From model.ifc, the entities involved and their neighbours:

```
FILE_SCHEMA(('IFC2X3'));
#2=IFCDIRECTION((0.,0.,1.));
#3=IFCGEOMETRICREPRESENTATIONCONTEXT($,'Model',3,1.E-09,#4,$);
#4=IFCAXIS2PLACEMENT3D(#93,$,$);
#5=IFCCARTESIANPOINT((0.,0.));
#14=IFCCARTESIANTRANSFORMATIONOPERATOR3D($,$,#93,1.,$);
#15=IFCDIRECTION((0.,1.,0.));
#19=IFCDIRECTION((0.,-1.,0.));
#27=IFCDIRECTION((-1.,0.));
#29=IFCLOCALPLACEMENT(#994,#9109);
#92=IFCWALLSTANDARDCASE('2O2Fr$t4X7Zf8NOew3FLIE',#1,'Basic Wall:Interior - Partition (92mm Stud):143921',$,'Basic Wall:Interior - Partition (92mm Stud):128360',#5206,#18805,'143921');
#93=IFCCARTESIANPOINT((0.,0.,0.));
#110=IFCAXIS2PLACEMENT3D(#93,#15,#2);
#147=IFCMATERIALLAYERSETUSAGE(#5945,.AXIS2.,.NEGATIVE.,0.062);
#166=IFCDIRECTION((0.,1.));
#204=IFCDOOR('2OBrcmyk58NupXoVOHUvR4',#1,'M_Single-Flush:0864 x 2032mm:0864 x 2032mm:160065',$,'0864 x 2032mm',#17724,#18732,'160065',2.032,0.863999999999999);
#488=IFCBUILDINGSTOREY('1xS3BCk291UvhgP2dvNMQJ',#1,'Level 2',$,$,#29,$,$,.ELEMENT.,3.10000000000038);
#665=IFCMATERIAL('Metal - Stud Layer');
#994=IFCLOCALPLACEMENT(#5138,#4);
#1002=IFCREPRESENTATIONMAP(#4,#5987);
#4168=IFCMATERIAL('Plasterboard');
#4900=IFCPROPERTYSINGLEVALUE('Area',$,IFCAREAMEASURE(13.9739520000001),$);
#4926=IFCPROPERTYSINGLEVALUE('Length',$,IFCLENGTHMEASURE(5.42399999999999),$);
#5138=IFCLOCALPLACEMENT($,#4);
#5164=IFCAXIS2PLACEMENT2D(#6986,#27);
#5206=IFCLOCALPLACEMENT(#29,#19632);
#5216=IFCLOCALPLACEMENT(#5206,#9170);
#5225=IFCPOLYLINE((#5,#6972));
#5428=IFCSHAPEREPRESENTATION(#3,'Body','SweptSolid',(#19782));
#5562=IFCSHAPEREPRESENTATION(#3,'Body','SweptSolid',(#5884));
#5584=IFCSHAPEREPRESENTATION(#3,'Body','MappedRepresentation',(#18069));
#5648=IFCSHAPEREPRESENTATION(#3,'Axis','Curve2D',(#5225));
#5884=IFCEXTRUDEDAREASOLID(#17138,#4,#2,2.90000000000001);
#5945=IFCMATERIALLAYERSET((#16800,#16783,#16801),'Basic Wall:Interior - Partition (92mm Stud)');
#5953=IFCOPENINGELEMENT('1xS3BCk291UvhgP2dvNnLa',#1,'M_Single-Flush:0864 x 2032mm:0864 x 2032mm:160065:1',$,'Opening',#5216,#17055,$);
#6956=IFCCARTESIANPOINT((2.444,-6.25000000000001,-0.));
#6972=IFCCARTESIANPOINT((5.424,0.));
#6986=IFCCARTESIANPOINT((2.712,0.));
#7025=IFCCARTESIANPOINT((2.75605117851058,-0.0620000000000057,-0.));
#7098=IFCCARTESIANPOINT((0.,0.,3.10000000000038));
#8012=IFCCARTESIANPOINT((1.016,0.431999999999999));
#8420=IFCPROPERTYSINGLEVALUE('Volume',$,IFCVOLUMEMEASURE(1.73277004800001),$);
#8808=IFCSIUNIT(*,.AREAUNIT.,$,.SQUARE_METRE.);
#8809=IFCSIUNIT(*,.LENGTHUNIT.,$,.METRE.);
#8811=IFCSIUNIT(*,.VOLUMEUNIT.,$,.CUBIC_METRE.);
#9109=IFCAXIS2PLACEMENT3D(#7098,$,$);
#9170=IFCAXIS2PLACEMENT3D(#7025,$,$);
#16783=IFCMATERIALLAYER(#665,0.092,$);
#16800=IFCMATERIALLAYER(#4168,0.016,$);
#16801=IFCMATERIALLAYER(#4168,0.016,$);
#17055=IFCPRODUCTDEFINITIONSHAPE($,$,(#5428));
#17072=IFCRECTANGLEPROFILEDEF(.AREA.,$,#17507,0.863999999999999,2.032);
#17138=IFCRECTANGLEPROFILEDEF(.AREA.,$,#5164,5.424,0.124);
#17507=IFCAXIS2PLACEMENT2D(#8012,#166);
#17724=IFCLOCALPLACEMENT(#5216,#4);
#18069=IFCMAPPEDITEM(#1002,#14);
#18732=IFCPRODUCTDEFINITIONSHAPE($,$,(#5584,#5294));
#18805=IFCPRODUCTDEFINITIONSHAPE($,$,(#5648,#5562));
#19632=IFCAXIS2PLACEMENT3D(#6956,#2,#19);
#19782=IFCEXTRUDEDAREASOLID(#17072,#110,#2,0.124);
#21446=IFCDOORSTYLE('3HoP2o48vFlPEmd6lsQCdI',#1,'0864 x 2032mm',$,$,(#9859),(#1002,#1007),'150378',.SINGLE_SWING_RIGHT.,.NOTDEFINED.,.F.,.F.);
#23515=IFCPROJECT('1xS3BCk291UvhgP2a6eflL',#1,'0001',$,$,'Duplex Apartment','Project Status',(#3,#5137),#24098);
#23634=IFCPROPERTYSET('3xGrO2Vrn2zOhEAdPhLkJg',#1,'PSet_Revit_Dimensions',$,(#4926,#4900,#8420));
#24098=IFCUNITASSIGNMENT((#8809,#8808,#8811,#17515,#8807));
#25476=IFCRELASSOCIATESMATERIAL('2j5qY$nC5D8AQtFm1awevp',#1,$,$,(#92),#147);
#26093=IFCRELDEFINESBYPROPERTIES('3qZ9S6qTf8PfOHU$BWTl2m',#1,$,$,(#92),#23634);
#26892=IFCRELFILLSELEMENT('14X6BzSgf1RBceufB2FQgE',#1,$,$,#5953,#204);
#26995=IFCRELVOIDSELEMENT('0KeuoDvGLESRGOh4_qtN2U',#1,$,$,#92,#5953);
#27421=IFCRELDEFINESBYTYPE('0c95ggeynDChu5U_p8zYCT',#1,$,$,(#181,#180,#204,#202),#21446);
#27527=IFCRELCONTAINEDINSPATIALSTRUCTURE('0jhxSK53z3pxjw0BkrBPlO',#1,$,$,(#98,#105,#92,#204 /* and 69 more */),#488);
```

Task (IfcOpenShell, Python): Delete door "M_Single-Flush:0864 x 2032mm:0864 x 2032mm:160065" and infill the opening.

```python
import ifcopenshell
import ifcopenshell.api.feature
import ifcopenshell.api.pset
import ifcopenshell.api.root
import ifcopenshell.geom
import ifcopenshell.util.element
import ifcopenshell.util.shape
import ifcopenshell.util.unit

model = ifcopenshell.open("model.ifc")
area_scale = ifcopenshell.util.unit.calculate_unit_scale(model, "AREAUNIT")
volume_scale = ifcopenshell.util.unit.calculate_unit_scale(model, "VOLUMEUNIT")
settings = ifcopenshell.geom.settings()


def volume(element):
    """Net volume in cubic metres, openings subtracted."""
    shape = ifcopenshell.geom.create_shape(settings, element)
    return ifcopenshell.util.shape.get_volume(shape.geometry)


door = model.by_guid("2OBrcmyk58NupXoVOHUvR4")
opening = door.FillsVoids[0].RelatingOpeningElement
wall = opening.VoidsElements[0].RelatingBuildingElement
before = volume(wall)

ifcopenshell.api.root.remove_product(model, product=door)
ifcopenshell.api.feature.remove_feature(model, feature=opening)

after = volume(wall)
thickness = 0.124  # wall thickness in metres

# Update the wall's stored quantities.
pset = model.by_id(ifcopenshell.util.element.get_pset(wall, "PSet_Revit_Dimensions", should_inherit=False)["id"])
ifcopenshell.api.pset.edit_pset(model, pset=pset, properties={
    "Area": model.create_entity("IfcAreaMeasure", after / thickness / area_scale),
    "Volume": model.create_entity("IfcVolumeMeasure", after / volume_scale),
})

print(f"wall volume {before:.3f} -> {after:.3f} m3")

model.write("model_v2.ifc")
```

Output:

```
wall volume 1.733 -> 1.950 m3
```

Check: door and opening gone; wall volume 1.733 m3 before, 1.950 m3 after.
